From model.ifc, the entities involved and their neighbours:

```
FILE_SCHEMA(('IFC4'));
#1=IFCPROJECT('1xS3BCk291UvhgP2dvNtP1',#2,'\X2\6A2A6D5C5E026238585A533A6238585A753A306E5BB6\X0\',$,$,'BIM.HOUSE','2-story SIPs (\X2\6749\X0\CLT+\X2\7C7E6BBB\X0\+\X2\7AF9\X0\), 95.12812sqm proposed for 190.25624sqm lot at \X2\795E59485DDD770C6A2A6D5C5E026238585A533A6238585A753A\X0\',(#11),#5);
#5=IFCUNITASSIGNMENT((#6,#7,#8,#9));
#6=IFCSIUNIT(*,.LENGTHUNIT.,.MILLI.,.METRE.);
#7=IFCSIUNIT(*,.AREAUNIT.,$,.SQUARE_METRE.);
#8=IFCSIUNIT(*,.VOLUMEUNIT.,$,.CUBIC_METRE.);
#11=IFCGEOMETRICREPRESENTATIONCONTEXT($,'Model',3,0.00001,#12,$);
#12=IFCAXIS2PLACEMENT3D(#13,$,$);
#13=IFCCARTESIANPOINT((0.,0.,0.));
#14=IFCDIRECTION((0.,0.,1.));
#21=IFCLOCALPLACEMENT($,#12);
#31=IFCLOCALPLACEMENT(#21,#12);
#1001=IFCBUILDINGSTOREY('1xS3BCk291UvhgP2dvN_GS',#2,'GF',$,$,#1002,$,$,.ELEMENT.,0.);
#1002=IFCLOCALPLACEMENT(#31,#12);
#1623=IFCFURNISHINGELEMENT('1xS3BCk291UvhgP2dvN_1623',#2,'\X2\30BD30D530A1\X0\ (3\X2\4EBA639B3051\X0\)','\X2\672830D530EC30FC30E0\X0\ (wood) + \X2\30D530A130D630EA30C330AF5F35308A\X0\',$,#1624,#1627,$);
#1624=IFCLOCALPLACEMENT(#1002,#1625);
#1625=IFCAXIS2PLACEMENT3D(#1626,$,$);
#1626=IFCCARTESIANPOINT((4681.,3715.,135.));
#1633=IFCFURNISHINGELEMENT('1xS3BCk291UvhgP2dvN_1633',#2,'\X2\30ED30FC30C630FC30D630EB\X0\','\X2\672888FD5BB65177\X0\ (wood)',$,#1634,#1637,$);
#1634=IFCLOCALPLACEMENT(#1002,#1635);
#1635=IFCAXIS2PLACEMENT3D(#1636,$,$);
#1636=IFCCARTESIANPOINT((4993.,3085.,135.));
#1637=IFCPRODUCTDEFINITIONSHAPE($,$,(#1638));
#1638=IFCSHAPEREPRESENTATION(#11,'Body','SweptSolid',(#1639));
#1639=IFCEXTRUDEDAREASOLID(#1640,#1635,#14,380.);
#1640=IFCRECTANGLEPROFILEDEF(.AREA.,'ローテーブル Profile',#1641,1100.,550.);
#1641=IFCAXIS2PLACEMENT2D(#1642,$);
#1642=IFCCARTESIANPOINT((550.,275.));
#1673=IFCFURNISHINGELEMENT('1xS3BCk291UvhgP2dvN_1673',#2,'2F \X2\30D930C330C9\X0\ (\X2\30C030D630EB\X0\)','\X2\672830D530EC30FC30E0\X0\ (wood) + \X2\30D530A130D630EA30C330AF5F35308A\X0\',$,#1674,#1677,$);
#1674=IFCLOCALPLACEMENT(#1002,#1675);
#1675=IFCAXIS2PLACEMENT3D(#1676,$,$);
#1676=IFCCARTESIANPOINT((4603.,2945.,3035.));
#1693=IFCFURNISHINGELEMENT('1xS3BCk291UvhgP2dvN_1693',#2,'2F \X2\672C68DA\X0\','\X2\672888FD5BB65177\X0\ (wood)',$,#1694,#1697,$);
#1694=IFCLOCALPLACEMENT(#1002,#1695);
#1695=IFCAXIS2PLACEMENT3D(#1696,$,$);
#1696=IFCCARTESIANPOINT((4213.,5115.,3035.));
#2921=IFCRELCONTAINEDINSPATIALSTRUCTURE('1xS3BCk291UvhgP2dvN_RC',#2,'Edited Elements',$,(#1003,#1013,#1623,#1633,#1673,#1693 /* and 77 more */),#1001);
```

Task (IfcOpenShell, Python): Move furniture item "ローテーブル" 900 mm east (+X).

```python
import ifcopenshell
import ifcopenshell.api.geometry
import ifcopenshell.util.placement

model = ifcopenshell.open("model.ifc")

item = model.by_guid("1xS3BCk291UvhgP2dvN_1633")
matrix = ifcopenshell.util.placement.get_local_placement(item.ObjectPlacement)
matrix[0, 3] += 900.0
ifcopenshell.api.geometry.edit_object_placement(model, product=item, matrix=matrix, is_si=False)

print(ifcopenshell.util.placement.get_local_placement(item.ObjectPlacement).round(3) + 0.0)

model.write("model_rev.ifc")
```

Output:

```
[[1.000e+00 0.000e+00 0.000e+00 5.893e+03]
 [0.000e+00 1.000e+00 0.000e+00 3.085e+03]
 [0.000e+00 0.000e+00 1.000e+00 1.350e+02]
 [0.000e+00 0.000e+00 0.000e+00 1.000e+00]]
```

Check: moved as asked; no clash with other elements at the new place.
